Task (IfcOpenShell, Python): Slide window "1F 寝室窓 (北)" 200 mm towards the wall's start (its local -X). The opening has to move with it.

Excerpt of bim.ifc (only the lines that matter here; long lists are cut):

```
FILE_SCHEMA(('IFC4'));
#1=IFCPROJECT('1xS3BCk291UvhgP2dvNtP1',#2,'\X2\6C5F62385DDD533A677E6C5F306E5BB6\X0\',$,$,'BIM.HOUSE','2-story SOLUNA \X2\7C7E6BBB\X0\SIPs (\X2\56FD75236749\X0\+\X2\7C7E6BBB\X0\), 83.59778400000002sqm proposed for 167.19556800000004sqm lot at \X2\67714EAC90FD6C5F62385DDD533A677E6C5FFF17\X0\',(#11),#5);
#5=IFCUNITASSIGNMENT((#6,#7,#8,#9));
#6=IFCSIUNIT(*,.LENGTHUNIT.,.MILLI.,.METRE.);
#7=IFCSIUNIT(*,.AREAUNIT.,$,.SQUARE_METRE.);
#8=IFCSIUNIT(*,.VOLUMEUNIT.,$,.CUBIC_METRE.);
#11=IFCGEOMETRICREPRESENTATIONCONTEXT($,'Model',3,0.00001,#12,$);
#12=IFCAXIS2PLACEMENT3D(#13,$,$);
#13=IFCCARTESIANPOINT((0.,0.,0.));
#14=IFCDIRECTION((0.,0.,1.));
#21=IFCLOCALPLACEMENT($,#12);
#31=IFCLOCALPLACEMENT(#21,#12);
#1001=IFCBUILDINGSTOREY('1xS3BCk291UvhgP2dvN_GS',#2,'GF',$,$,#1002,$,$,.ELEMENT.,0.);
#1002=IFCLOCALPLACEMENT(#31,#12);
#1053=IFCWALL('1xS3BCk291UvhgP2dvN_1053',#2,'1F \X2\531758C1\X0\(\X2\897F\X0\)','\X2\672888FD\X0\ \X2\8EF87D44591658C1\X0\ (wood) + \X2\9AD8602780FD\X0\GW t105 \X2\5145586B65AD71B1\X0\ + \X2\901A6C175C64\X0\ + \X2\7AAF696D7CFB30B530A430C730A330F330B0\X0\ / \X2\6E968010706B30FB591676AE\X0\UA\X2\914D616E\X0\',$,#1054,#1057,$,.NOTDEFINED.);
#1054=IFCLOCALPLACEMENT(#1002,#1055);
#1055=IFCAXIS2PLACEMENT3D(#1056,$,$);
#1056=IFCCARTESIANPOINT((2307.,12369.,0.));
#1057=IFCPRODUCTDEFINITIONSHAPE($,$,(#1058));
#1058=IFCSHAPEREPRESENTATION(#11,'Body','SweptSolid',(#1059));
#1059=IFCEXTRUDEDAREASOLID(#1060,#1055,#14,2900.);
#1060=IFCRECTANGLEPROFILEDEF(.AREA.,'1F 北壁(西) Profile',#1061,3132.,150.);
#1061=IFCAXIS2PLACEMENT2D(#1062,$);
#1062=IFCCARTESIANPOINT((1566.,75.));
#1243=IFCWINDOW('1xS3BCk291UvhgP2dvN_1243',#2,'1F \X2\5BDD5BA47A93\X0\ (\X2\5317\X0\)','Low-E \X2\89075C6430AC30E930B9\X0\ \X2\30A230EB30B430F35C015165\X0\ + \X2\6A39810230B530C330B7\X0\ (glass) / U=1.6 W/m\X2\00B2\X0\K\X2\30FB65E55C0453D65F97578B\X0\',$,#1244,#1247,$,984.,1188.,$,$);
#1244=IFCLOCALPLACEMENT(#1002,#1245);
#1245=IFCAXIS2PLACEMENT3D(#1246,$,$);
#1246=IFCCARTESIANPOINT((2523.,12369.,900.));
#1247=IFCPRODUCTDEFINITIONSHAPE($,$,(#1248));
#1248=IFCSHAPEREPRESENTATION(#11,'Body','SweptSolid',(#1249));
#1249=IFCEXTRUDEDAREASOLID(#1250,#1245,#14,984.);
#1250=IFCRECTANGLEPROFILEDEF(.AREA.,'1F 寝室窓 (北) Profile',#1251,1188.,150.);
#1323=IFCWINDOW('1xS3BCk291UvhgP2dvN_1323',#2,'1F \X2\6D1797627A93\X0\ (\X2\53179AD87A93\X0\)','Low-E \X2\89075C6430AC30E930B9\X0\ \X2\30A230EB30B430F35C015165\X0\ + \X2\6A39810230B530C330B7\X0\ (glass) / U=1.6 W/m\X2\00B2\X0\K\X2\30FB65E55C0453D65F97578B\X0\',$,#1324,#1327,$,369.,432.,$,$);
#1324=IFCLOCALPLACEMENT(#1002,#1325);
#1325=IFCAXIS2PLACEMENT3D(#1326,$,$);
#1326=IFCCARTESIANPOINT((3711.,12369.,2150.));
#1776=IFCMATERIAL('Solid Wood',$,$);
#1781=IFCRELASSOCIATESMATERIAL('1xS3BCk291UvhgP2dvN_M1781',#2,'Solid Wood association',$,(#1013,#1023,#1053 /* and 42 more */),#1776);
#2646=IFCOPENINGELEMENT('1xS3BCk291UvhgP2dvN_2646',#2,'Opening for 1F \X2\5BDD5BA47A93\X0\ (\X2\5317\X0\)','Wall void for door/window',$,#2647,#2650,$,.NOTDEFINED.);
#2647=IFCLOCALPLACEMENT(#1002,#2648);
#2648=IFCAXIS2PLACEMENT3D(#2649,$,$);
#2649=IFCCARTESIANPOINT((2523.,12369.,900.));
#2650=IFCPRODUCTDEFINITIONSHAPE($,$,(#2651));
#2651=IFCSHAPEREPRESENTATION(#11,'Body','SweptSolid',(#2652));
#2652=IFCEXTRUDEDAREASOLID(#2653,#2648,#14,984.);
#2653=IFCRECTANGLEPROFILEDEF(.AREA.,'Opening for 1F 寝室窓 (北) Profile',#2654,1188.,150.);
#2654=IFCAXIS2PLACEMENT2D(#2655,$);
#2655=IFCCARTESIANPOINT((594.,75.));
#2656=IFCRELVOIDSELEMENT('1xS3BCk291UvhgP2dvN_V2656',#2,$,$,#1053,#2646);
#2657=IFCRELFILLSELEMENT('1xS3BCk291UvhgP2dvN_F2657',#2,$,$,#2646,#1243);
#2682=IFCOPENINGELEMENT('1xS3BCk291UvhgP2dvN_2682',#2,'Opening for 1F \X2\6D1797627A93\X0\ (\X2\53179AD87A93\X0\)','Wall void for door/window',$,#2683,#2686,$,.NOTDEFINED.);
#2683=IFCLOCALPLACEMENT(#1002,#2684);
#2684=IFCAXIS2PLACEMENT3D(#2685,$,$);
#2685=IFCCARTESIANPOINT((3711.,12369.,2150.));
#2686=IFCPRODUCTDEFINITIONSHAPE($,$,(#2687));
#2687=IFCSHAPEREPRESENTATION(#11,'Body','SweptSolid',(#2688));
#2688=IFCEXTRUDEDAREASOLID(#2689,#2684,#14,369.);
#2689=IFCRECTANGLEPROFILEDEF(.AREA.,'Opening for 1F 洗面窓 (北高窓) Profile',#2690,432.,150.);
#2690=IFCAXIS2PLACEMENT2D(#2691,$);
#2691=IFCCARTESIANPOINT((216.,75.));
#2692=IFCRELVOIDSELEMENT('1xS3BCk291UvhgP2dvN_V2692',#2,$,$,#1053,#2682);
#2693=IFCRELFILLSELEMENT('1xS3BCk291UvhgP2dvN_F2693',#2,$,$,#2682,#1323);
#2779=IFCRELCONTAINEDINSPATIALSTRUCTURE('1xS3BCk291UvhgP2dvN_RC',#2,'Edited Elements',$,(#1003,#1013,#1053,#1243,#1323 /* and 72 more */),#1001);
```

```python
import ifcopenshell
import ifcopenshell.api.geometry
import ifcopenshell.util.placement

model = ifcopenshell.open("bim.ifc")

window = model.by_id(1243)
opening = window.FillsVoids[0].RelatingOpeningElement
wall = opening.VoidsElements[0].RelatingBuildingElement

wall_matrix = ifcopenshell.util.placement.get_local_placement(wall.ObjectPlacement)
shift = wall_matrix[:3, 0] * -200.0
before = ifcopenshell.util.placement.get_local_placement(window.ObjectPlacement)[:3, 3].copy()

# The window is not placed relative to its opening, so move both.
for product in (opening, window):
    matrix = ifcopenshell.util.placement.get_local_placement(product.ObjectPlacement)
    matrix[:3, 3] += shift
    ifcopenshell.api.geometry.edit_object_placement(model, product=product, matrix=matrix, is_si=False)

after = ifcopenshell.util.placement.get_local_placement(window.ObjectPlacement)[:3, 3]
print("window moved by", (after - before).round(3) + 0.0)

model.write("bim_updated.ifc")
```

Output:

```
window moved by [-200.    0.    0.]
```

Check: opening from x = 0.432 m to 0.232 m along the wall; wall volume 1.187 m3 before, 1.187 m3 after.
